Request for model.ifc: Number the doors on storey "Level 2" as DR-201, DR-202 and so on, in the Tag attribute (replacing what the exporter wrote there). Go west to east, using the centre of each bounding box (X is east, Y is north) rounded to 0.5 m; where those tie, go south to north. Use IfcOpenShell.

First a look at what the model holds.

```python
import ifcopenshell
import ifcopenshell.util.element
import ifcopenshell.util.placement

model = ifcopenshell.open("model.ifc")
print(model.schema)
storey = next(s for s in model.by_type("IfcBuildingStorey") if s.Name == "Level 2")
doors = [e for e in ifcopenshell.util.element.get_decomposition(storey) if e.is_a("IfcDoor")]
for e in sorted(doors, key=lambda e: e.id()):
    origin = ifcopenshell.util.placement.get_local_placement(e.ObjectPlacement)[:3, 3]
    print(e.id(), e.Tag, e.Name, origin.round(2) + 0.0, sep=" | ")
```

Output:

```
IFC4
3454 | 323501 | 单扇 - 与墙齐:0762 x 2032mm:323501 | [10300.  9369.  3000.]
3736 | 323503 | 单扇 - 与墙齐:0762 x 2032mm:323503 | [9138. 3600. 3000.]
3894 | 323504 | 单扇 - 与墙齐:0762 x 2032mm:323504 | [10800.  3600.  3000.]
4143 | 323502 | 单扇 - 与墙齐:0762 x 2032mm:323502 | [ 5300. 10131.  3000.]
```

```python
import ifcopenshell
import ifcopenshell.geom
import ifcopenshell.util.element
import ifcopenshell.util.shape

model = ifcopenshell.open("model.ifc")
settings = ifcopenshell.geom.settings()
settings.set("use-world-coords", True)


def centre(element):
    shape = ifcopenshell.geom.create_shape(settings, element)
    return ifcopenshell.util.shape.get_bbox_centroid(shape.geometry)


storey = next(s for s in model.by_type("IfcBuildingStorey") if s.Name == "Level 2")
doors = [e for e in ifcopenshell.util.element.get_decomposition(storey) if e.is_a("IfcDoor")]

# Insertion points can sit at a corner or the storey origin, so sort by the geometry (in metres).
centres = {e: centre(e) for e in doors}
doors.sort(key=lambda e: (round(centres[e][0] / 0.5), centres[e][1]))

for i, e in enumerate(doors, start=1):
    number = f"DR-2{i:02d}"
    e.Tag = number
    print(e.id(), number)

model.write("model_v2.ifc")
```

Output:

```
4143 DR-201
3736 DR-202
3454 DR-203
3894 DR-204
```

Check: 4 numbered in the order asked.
